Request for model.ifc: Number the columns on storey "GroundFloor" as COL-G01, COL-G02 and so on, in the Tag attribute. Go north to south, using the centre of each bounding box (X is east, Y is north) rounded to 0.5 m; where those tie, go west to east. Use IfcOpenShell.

First a look at what the model holds.

```python
import ifcopenshell
import ifcopenshell.util.element
import ifcopenshell.util.placement

model = ifcopenshell.open("model.ifc")
print(model.schema)
storey = next(s for s in model.by_type("IfcBuildingStorey") if s.Name == "GroundFloor")
columns = [e for e in ifcopenshell.util.element.get_decomposition(storey) if e.is_a("IfcColumn")]
for e in sorted(columns, key=lambda e: e.id()):
    origin = ifcopenshell.util.placement.get_local_placement(e.ObjectPlacement)[:3, 3]
    print(e.id(), e.Tag, e.Name, origin.round(2) + 0.0, sep=" | ")
```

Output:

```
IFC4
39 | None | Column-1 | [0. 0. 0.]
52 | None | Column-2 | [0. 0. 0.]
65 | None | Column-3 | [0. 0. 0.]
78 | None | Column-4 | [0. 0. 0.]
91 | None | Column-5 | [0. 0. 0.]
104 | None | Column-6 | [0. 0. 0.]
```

```python
import ifcopenshell
import ifcopenshell.geom
import ifcopenshell.util.element
import ifcopenshell.util.shape

model = ifcopenshell.open("model.ifc")
settings = ifcopenshell.geom.settings()
settings.set("use-world-coords", True)


def centre(element):
    shape = ifcopenshell.geom.create_shape(settings, element)
    return ifcopenshell.util.shape.get_bbox_centroid(shape.geometry)


storey = next(s for s in model.by_type("IfcBuildingStorey") if s.Name == "GroundFloor")
columns = [e for e in ifcopenshell.util.element.get_decomposition(storey) if e.is_a("IfcColumn")]

# Insertion points can sit at a corner or the storey origin, so sort by the geometry (in metres).
centres = {e: centre(e) for e in columns}
columns.sort(key=lambda e: (-round(centres[e][1] / 0.5), centres[e][0]))

for i, e in enumerate(columns, start=1):
    number = f"COL-G{i:02d}"
    e.Tag = number
    print(e.id(), number)

model.write("model-out.ifc")
```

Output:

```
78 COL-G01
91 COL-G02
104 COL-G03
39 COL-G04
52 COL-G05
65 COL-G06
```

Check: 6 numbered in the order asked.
